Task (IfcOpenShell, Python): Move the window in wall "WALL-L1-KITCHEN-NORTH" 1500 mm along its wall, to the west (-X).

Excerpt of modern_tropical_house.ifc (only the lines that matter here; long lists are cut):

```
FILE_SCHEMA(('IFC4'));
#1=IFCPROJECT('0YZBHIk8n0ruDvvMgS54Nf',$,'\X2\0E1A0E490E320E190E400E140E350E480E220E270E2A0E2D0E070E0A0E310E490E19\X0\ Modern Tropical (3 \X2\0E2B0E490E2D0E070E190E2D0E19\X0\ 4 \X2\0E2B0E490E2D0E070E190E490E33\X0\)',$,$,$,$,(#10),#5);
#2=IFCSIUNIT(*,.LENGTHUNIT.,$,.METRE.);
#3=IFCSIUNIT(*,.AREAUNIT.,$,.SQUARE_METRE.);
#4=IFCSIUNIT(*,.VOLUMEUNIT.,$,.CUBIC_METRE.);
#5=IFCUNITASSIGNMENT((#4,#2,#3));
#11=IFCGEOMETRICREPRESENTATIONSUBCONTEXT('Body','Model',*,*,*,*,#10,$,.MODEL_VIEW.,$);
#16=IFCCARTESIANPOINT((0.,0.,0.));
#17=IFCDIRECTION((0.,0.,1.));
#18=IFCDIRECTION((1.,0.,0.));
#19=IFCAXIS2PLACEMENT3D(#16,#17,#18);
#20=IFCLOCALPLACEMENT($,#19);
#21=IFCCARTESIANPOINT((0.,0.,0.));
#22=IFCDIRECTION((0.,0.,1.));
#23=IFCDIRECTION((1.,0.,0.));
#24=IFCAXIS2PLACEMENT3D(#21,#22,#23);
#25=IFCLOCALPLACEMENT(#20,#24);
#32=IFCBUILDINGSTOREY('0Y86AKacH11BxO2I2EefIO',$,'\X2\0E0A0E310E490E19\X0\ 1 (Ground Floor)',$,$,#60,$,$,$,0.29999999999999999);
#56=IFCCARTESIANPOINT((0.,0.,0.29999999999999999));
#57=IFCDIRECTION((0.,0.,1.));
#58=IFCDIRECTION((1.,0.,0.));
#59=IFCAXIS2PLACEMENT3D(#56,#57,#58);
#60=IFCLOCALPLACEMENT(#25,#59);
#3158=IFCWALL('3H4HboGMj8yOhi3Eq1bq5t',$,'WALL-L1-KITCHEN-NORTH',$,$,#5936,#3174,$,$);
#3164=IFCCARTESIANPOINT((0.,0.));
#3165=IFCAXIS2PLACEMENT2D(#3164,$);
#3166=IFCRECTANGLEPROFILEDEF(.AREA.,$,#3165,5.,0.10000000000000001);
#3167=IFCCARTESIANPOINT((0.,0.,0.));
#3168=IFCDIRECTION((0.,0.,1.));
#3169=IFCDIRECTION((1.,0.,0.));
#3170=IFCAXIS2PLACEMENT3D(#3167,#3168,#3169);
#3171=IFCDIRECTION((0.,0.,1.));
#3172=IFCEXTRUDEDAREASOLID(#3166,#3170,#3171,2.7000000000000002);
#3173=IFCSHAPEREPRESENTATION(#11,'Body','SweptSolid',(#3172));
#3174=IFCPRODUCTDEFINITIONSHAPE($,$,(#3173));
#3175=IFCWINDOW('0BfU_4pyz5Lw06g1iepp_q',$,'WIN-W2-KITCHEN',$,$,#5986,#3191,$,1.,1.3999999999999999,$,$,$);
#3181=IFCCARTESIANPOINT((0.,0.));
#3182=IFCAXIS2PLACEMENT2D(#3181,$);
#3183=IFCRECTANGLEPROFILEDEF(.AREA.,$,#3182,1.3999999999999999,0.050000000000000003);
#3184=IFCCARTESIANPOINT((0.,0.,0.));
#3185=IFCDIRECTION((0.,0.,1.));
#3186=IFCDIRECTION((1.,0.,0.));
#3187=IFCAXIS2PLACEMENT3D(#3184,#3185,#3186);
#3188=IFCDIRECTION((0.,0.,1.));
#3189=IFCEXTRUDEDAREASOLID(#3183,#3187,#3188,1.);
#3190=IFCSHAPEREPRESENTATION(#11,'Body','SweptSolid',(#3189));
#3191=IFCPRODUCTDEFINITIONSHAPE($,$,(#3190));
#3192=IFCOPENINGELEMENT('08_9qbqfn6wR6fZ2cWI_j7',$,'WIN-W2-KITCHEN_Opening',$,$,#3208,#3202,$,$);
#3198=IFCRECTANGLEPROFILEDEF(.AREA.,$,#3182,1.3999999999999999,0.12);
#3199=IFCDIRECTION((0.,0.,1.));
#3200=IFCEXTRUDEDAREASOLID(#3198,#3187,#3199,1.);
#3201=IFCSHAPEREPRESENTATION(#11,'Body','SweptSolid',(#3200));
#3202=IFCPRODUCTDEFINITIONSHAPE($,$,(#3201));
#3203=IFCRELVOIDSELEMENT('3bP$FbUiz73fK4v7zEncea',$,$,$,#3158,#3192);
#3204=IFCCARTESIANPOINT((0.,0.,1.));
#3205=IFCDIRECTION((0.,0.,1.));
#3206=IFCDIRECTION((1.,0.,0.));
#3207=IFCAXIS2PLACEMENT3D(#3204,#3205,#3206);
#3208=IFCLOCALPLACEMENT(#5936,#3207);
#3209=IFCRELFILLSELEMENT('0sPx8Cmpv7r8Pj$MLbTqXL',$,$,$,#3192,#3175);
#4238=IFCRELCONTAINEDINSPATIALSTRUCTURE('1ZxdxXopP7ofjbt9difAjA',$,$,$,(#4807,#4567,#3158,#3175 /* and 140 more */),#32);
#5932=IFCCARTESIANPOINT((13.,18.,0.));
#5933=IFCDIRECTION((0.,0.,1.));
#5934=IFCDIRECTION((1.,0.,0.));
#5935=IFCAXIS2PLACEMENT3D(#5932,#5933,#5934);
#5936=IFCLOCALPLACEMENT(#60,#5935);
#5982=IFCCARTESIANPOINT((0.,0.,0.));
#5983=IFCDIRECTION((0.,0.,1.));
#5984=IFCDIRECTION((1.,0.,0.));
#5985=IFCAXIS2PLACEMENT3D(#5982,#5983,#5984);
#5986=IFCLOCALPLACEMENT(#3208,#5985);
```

```python
import ifcopenshell
import ifcopenshell.api.geometry
import ifcopenshell.util.placement

model = ifcopenshell.open("modern_tropical_house.ifc")

window = model.by_id(3175)
opening = window.FillsVoids[0].RelatingOpeningElement
wall = opening.VoidsElements[0].RelatingBuildingElement

wall_matrix = ifcopenshell.util.placement.get_local_placement(wall.ObjectPlacement)
shift = wall_matrix[:3, 0] * -1.5
before = ifcopenshell.util.placement.get_local_placement(window.ObjectPlacement)[:3, 3].copy()

# The window is placed relative to its opening, so it follows when the opening moves.
matrix = ifcopenshell.util.placement.get_local_placement(opening.ObjectPlacement)
matrix[:3, 3] += shift
ifcopenshell.api.geometry.edit_object_placement(
    model, product=opening, matrix=matrix, is_si=False, should_transform_children=True
)

after = ifcopenshell.util.placement.get_local_placement(window.ObjectPlacement)[:3, 3]
print("window moved by", (after - before).round(3) + 0.0)

model.write("modern_tropical_house_rev.ifc")
```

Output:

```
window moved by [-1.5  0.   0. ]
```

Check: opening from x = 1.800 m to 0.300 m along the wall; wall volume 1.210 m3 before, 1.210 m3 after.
